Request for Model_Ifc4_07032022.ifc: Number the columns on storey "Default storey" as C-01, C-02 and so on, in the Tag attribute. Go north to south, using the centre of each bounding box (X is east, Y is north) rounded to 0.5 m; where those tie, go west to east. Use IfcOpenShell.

First a look at what the model holds.

```python
import ifcopenshell
import ifcopenshell.util.element
import ifcopenshell.util.placement

model = ifcopenshell.open("Model_Ifc4_07032022.ifc")
print(model.schema)
storey = next(s for s in model.by_type("IfcBuildingStorey") if s.Name == "Default storey")
columns = [e for e in ifcopenshell.util.element.get_decomposition(storey) if e.is_a("IfcColumn")]
for e in sorted(columns, key=lambda e: e.id()):
    origin = ifcopenshell.util.placement.get_local_placement(e.ObjectPlacement)[:3, 3]
    print(e.id(), e.Tag, e.Name, origin.round(2) + 0.0, sep=" | ")
```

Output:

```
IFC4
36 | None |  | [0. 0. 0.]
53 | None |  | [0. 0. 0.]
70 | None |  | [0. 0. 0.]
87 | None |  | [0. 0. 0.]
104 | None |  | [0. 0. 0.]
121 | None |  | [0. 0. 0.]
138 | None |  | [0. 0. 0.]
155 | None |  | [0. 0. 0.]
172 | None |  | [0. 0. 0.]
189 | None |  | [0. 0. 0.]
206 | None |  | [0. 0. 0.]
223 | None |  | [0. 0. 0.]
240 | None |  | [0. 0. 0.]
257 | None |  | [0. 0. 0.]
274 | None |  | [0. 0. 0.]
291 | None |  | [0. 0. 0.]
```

```python
import ifcopenshell
import ifcopenshell.geom
import ifcopenshell.util.element
import ifcopenshell.util.shape

model = ifcopenshell.open("Model_Ifc4_07032022.ifc")
settings = ifcopenshell.geom.settings()
settings.set("use-world-coords", True)


def centre(element):
    shape = ifcopenshell.geom.create_shape(settings, element)
    return ifcopenshell.util.shape.get_bbox_centroid(shape.geometry)


storey = next(s for s in model.by_type("IfcBuildingStorey") if s.Name == "Default storey")
columns = [e for e in ifcopenshell.util.element.get_decomposition(storey) if e.is_a("IfcColumn")]

# Insertion points can sit at a corner or the storey origin, so sort by the geometry (in metres).
centres = {e: centre(e) for e in columns}
columns.sort(key=lambda e: (-round(centres[e][1] / 0.5), centres[e][0]))

for i, e in enumerate(columns, start=1):
    number = f"C-{i:02d}"
    e.Tag = number
    print(e.id(), number)

model.write("Model_Ifc4_07032022_v2.ifc")
```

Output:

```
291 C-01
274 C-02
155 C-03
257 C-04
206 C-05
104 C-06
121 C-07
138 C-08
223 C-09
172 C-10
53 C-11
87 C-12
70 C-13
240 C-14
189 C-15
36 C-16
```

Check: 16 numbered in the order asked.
